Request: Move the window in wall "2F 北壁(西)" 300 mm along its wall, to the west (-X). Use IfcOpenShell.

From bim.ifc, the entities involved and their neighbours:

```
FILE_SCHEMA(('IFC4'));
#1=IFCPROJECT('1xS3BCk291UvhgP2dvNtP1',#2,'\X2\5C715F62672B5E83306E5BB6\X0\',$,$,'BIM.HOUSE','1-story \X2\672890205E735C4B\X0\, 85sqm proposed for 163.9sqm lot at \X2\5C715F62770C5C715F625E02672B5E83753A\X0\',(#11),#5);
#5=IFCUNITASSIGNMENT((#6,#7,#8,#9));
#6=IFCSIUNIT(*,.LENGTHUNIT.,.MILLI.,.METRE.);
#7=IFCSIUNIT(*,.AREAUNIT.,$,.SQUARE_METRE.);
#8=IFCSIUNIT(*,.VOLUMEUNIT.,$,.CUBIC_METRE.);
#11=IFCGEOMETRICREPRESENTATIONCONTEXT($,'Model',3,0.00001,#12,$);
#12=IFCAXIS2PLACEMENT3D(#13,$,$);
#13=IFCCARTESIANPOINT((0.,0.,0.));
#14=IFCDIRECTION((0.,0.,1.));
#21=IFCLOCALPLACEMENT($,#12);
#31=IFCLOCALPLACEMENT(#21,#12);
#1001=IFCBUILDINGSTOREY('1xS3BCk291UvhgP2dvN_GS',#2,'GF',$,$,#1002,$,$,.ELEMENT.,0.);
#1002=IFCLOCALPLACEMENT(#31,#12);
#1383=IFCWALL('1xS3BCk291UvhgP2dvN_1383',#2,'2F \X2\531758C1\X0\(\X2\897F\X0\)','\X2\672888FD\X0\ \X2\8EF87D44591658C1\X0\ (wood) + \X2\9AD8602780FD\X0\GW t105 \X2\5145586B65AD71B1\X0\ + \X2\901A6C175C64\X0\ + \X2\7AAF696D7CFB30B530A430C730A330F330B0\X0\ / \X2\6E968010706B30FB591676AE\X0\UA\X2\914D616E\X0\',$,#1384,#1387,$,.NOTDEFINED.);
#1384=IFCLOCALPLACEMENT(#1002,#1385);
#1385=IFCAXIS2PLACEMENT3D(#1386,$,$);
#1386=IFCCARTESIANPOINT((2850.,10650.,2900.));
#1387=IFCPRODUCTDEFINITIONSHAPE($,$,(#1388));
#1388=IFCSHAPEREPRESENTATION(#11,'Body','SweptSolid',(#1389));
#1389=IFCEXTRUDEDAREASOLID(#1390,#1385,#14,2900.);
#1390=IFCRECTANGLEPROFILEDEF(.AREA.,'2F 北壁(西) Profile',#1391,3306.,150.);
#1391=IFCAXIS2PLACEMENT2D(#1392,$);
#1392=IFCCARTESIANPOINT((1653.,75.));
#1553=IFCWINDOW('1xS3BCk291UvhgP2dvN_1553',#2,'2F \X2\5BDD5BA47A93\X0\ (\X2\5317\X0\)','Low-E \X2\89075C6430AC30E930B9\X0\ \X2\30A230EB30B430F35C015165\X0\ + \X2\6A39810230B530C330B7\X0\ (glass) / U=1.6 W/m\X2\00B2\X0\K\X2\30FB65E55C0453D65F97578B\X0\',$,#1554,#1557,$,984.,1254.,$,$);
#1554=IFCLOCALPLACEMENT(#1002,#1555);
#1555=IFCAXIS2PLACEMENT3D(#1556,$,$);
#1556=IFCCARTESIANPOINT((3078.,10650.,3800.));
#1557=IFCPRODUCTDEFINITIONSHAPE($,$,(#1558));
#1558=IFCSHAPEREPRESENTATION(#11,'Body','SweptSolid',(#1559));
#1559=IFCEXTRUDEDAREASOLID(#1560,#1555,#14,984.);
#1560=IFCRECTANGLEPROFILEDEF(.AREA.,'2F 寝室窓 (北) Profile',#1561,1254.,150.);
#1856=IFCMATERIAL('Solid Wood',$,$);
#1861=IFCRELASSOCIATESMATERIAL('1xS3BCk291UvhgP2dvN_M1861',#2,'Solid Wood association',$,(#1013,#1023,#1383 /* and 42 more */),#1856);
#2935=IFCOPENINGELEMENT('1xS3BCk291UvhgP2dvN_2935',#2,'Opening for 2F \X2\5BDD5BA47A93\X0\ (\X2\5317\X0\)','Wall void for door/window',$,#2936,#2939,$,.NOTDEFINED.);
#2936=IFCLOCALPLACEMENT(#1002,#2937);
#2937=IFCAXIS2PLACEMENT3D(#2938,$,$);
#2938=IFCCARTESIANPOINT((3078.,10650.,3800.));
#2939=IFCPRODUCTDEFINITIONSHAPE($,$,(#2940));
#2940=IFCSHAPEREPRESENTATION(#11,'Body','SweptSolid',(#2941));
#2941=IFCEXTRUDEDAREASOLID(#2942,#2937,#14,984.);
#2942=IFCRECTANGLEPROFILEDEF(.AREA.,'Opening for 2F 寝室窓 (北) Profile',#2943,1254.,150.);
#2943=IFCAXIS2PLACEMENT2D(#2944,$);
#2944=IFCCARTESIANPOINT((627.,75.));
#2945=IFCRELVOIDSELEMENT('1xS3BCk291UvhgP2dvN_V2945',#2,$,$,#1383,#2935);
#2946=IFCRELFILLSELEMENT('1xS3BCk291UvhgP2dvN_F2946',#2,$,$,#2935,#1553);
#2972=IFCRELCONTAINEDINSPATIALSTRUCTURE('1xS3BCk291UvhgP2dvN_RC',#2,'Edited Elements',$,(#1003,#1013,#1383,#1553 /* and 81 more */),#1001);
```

```python
import ifcopenshell
import ifcopenshell.api.geometry
import ifcopenshell.util.placement

model = ifcopenshell.open("bim.ifc")

window = model.by_id(1553)
opening = window.FillsVoids[0].RelatingOpeningElement
wall = opening.VoidsElements[0].RelatingBuildingElement

wall_matrix = ifcopenshell.util.placement.get_local_placement(wall.ObjectPlacement)
shift = wall_matrix[:3, 0] * -300.0
before = ifcopenshell.util.placement.get_local_placement(window.ObjectPlacement)[:3, 3].copy()

# The window is not placed relative to its opening, so move both.
for product in (opening, window):
    matrix = ifcopenshell.util.placement.get_local_placement(product.ObjectPlacement)
    matrix[:3, 3] += shift
    ifcopenshell.api.geometry.edit_object_placement(model, product=product, matrix=matrix, is_si=False)

after = ifcopenshell.util.placement.get_local_placement(window.ObjectPlacement)[:3, 3]
print("window moved by", (after - before).round(3) + 0.0)

model.write("bim_edited.ifc")
```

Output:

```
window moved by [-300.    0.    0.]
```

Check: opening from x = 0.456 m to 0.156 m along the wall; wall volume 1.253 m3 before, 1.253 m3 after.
